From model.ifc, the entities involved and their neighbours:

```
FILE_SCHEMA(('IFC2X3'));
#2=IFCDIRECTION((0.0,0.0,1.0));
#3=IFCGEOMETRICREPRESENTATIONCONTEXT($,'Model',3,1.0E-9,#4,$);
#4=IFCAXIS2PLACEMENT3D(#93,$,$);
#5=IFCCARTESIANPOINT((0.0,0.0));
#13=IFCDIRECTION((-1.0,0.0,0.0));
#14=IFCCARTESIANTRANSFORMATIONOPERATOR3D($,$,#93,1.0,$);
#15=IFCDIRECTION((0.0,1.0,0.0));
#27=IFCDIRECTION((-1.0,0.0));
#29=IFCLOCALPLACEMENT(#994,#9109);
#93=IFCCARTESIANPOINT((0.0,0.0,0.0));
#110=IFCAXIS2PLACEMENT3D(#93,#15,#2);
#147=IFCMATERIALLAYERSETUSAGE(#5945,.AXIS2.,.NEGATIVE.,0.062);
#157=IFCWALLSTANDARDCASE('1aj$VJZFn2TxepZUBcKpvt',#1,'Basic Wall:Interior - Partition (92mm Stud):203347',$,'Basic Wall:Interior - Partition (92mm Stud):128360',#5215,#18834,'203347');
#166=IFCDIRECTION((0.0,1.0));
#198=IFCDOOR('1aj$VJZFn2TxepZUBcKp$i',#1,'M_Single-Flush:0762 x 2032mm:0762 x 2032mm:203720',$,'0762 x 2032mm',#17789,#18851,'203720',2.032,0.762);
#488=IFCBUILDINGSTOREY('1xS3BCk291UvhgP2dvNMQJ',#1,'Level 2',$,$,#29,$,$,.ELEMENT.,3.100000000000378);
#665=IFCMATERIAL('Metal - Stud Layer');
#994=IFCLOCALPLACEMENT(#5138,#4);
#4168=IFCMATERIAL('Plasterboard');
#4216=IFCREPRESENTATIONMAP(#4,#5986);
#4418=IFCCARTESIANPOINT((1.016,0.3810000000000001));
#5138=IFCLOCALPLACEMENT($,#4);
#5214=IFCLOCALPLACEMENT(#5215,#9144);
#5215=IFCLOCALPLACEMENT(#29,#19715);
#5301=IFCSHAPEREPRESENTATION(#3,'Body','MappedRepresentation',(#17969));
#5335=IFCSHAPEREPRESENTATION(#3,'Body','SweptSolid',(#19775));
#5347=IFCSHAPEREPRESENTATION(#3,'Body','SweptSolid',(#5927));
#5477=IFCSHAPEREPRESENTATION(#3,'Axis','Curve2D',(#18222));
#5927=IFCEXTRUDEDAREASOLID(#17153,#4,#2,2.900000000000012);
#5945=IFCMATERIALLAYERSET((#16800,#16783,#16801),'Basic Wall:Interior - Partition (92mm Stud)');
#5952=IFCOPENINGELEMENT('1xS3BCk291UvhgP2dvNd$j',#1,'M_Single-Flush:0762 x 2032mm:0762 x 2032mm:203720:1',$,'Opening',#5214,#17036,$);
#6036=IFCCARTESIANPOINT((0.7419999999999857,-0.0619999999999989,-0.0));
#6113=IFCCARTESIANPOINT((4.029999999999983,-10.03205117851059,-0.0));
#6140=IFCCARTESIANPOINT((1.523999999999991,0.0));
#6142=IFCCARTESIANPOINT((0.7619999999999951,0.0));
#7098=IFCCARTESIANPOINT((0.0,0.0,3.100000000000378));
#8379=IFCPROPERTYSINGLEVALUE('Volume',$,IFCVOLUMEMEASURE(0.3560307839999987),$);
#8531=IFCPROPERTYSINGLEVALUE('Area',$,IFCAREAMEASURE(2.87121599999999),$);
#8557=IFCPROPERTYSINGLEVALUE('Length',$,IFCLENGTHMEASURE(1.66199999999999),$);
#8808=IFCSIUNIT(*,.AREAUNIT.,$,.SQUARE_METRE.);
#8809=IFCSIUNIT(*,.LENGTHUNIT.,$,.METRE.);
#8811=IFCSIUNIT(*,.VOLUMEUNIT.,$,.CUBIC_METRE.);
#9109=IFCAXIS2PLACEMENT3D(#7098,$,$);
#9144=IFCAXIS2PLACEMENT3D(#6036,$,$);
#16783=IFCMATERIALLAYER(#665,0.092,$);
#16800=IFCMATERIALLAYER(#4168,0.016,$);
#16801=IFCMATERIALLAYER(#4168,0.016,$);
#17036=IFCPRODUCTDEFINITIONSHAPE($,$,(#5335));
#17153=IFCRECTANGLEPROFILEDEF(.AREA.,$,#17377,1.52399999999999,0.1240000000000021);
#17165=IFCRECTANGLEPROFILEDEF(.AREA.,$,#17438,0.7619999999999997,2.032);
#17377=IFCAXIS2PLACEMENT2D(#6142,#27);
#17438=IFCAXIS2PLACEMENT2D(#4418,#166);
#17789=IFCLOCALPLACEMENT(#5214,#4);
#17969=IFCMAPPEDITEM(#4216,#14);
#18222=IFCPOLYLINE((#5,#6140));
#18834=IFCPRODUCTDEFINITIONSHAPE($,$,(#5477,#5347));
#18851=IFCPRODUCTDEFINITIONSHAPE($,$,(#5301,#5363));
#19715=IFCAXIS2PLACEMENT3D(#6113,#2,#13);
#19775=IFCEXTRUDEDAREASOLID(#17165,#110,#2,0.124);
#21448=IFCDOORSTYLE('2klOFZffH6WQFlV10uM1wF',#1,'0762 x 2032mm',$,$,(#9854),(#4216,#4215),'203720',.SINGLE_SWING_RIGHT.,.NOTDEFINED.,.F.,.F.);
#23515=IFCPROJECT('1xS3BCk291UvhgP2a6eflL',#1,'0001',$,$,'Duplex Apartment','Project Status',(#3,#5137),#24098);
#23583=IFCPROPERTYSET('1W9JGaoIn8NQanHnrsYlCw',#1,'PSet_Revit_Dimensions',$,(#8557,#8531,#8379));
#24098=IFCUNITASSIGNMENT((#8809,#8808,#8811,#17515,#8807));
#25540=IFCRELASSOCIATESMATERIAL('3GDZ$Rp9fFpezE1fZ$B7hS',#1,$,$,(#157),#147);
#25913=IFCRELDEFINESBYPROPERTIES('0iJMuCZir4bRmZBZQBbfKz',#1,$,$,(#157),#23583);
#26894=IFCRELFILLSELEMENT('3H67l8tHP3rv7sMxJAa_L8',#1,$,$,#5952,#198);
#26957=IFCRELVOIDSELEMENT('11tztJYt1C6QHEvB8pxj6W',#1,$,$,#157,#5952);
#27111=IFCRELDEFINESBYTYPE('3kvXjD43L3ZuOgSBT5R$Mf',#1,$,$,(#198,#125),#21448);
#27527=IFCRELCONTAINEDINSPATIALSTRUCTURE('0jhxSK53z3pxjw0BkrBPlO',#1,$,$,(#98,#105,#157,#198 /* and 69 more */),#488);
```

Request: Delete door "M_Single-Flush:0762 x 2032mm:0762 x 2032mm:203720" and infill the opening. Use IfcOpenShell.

```python
import ifcopenshell
import ifcopenshell.api.feature
import ifcopenshell.api.pset
import ifcopenshell.api.root
import ifcopenshell.geom
import ifcopenshell.util.element
import ifcopenshell.util.shape
import ifcopenshell.util.unit

model = ifcopenshell.open("model.ifc")
area_scale = ifcopenshell.util.unit.calculate_unit_scale(model, "AREAUNIT")
volume_scale = ifcopenshell.util.unit.calculate_unit_scale(model, "VOLUMEUNIT")
settings = ifcopenshell.geom.settings()


def volume(element):
    """Net volume in cubic metres, openings subtracted."""
    shape = ifcopenshell.geom.create_shape(settings, element)
    return ifcopenshell.util.shape.get_volume(shape.geometry)


door = model.by_guid("1aj$VJZFn2TxepZUBcKp$i")
opening = door.FillsVoids[0].RelatingOpeningElement
wall = opening.VoidsElements[0].RelatingBuildingElement
before = volume(wall)

ifcopenshell.api.root.remove_product(model, product=door)
ifcopenshell.api.feature.remove_feature(model, feature=opening)

after = volume(wall)
thickness = 0.124  # wall thickness in metres

# Update the wall's stored quantities.
pset = model.by_id(ifcopenshell.util.element.get_pset(wall, "PSet_Revit_Dimensions", should_inherit=False)["id"])
ifcopenshell.api.pset.edit_pset(model, pset=pset, properties={
    "Area": model.create_entity("IfcAreaMeasure", after / thickness / area_scale),
    "Volume": model.create_entity("IfcVolumeMeasure", after / volume_scale),
})

print(f"wall volume {before:.3f} -> {after:.3f} m3")

model.write("model_edited.ifc")
```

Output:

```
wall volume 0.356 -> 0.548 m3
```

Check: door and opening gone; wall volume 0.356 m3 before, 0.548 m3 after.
